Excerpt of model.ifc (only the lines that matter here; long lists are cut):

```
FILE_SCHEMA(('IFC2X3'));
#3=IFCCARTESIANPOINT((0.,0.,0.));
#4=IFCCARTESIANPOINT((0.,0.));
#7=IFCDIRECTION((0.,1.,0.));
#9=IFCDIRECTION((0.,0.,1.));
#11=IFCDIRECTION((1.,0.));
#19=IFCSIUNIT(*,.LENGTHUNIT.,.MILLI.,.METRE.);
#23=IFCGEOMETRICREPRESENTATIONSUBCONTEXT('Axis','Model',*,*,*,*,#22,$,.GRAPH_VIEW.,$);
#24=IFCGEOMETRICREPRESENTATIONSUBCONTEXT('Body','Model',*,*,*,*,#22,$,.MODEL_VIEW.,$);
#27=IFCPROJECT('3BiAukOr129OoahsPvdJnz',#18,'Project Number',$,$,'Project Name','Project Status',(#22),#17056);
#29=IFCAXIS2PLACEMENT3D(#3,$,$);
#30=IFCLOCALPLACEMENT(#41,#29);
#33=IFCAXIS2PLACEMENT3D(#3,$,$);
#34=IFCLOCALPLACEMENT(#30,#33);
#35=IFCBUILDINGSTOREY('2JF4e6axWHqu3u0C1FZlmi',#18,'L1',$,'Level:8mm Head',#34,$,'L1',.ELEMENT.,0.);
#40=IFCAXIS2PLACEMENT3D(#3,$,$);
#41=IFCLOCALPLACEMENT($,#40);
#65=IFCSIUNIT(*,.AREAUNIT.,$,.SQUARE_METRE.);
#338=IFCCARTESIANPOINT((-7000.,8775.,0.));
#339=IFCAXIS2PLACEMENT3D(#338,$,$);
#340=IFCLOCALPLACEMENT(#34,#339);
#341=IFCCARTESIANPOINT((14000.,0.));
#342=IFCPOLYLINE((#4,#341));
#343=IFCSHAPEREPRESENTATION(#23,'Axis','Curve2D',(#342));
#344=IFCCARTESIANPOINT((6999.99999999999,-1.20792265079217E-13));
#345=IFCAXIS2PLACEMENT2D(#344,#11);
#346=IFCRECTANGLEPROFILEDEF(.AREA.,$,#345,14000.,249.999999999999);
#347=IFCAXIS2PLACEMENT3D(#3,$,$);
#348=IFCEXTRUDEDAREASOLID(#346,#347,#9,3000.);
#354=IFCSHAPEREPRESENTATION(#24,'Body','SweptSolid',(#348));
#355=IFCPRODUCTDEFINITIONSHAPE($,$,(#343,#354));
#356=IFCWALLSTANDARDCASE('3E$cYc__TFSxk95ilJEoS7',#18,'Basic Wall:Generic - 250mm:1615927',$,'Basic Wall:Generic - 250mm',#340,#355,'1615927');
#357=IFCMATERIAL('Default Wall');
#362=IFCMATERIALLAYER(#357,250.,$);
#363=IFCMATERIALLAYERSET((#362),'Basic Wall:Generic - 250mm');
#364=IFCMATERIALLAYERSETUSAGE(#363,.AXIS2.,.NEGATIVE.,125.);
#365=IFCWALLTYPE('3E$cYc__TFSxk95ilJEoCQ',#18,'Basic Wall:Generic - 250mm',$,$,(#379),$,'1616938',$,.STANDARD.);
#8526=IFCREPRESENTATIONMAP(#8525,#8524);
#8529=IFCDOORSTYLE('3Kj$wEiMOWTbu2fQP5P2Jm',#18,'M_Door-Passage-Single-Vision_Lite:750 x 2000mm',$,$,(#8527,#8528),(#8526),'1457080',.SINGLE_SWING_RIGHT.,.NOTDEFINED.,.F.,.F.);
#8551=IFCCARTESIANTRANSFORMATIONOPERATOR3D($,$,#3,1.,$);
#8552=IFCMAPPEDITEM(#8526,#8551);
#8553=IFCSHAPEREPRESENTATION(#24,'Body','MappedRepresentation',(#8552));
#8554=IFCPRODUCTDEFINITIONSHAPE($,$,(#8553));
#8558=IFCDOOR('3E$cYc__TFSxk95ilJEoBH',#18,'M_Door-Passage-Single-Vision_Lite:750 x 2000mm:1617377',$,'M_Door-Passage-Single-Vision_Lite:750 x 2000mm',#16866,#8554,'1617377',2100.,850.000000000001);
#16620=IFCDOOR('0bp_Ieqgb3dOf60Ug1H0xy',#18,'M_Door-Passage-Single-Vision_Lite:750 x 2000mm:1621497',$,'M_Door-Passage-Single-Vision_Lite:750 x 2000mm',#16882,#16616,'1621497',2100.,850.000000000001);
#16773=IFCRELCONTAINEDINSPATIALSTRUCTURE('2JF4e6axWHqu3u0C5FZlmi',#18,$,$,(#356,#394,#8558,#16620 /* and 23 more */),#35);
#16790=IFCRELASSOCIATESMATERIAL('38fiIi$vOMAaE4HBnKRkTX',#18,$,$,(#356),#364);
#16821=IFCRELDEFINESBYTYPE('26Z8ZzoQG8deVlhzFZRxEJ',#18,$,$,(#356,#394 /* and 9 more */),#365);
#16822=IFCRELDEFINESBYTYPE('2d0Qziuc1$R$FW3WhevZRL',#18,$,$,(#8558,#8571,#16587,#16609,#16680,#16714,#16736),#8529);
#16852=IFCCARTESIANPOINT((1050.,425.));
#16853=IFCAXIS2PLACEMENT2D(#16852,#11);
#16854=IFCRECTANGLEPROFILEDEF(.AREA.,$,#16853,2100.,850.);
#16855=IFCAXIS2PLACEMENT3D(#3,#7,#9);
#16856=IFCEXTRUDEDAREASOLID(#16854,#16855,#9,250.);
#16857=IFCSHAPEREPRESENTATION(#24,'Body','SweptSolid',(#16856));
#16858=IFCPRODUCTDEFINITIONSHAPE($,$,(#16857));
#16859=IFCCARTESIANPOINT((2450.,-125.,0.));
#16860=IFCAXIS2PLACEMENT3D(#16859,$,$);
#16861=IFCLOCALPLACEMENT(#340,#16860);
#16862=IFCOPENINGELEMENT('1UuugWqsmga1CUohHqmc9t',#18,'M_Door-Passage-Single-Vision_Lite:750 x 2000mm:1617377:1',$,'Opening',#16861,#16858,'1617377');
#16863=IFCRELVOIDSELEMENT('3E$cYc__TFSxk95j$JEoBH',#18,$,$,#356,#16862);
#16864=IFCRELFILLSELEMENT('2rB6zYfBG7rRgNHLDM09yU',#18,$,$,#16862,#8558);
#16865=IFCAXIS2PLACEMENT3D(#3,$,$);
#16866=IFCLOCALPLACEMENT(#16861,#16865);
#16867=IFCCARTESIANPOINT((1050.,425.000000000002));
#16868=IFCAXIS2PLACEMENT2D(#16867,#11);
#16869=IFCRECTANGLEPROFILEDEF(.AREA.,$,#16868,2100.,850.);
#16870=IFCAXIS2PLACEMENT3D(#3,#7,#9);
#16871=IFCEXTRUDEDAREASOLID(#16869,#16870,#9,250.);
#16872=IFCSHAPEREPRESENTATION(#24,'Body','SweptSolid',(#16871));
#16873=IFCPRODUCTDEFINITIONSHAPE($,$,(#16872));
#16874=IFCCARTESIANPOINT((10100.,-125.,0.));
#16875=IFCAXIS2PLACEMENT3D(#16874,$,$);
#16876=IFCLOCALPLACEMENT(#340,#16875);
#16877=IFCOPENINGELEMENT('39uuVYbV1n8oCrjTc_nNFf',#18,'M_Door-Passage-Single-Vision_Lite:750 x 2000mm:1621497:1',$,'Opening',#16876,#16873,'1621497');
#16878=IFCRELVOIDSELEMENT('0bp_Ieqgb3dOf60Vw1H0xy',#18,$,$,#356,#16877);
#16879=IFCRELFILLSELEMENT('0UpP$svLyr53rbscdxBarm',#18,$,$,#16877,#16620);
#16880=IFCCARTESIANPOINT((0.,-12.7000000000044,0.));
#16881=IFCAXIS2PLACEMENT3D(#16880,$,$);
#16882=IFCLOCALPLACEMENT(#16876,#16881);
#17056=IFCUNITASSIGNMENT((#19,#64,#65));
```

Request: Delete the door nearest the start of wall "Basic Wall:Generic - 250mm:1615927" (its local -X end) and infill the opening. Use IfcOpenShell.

```python
import ifcopenshell
import ifcopenshell.api.feature
import ifcopenshell.api.root
import ifcopenshell.geom
import ifcopenshell.util.shape

model = ifcopenshell.open("model.ifc")
settings = ifcopenshell.geom.settings()


def volume(element):
    """Net volume in cubic metres, openings subtracted."""
    shape = ifcopenshell.geom.create_shape(settings, element)
    return ifcopenshell.util.shape.get_volume(shape.geometry)


door = model.by_id(8558)
opening = door.FillsVoids[0].RelatingOpeningElement
wall = opening.VoidsElements[0].RelatingBuildingElement
before = volume(wall)

ifcopenshell.api.root.remove_product(model, product=door)
ifcopenshell.api.feature.remove_feature(model, feature=opening)

after = volume(wall)

print(f"wall volume {before:.3f} -> {after:.3f} m3")

model.write("model_rev.ifc")
```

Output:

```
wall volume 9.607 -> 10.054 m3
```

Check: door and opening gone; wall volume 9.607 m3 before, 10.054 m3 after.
